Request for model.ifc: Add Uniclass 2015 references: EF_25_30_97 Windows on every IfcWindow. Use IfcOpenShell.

First a look at what the model holds.

```python
import ifcopenshell

model = ifcopenshell.open("model.ifc")
print(model.schema)
print("classifications:", [c.Name for c in model.by_type("IfcClassification")])
for ifc_class in ("IfcDoor", "IfcRoof", "IfcStair", "IfcWall", "IfcWindow"):
    print(ifc_class, len(model.by_type(ifc_class)))
```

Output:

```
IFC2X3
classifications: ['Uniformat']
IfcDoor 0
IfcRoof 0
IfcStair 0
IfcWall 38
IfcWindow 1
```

```python
import ifcopenshell
import ifcopenshell.api.classification

model = ifcopenshell.open("model.ifc")

# IFC2X3 requires Source and Edition and has no link from the project to the system.
system = model.create_entity("IfcClassification", Source="NBS", Edition="2015", Name="Uniclass 2015")

codes = {
    "IfcWindow": ("EF_25_30_97", "Windows"),
}
for ifc_class, (code, name) in codes.items():
    products = model.by_type(ifc_class)
    ifcopenshell.api.classification.add_reference(
        model, products=products, classification=system, identification=code, name=name
    )
    print(code, len(products))

model.write("model_updated.ifc")
```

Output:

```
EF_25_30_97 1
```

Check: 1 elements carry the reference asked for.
